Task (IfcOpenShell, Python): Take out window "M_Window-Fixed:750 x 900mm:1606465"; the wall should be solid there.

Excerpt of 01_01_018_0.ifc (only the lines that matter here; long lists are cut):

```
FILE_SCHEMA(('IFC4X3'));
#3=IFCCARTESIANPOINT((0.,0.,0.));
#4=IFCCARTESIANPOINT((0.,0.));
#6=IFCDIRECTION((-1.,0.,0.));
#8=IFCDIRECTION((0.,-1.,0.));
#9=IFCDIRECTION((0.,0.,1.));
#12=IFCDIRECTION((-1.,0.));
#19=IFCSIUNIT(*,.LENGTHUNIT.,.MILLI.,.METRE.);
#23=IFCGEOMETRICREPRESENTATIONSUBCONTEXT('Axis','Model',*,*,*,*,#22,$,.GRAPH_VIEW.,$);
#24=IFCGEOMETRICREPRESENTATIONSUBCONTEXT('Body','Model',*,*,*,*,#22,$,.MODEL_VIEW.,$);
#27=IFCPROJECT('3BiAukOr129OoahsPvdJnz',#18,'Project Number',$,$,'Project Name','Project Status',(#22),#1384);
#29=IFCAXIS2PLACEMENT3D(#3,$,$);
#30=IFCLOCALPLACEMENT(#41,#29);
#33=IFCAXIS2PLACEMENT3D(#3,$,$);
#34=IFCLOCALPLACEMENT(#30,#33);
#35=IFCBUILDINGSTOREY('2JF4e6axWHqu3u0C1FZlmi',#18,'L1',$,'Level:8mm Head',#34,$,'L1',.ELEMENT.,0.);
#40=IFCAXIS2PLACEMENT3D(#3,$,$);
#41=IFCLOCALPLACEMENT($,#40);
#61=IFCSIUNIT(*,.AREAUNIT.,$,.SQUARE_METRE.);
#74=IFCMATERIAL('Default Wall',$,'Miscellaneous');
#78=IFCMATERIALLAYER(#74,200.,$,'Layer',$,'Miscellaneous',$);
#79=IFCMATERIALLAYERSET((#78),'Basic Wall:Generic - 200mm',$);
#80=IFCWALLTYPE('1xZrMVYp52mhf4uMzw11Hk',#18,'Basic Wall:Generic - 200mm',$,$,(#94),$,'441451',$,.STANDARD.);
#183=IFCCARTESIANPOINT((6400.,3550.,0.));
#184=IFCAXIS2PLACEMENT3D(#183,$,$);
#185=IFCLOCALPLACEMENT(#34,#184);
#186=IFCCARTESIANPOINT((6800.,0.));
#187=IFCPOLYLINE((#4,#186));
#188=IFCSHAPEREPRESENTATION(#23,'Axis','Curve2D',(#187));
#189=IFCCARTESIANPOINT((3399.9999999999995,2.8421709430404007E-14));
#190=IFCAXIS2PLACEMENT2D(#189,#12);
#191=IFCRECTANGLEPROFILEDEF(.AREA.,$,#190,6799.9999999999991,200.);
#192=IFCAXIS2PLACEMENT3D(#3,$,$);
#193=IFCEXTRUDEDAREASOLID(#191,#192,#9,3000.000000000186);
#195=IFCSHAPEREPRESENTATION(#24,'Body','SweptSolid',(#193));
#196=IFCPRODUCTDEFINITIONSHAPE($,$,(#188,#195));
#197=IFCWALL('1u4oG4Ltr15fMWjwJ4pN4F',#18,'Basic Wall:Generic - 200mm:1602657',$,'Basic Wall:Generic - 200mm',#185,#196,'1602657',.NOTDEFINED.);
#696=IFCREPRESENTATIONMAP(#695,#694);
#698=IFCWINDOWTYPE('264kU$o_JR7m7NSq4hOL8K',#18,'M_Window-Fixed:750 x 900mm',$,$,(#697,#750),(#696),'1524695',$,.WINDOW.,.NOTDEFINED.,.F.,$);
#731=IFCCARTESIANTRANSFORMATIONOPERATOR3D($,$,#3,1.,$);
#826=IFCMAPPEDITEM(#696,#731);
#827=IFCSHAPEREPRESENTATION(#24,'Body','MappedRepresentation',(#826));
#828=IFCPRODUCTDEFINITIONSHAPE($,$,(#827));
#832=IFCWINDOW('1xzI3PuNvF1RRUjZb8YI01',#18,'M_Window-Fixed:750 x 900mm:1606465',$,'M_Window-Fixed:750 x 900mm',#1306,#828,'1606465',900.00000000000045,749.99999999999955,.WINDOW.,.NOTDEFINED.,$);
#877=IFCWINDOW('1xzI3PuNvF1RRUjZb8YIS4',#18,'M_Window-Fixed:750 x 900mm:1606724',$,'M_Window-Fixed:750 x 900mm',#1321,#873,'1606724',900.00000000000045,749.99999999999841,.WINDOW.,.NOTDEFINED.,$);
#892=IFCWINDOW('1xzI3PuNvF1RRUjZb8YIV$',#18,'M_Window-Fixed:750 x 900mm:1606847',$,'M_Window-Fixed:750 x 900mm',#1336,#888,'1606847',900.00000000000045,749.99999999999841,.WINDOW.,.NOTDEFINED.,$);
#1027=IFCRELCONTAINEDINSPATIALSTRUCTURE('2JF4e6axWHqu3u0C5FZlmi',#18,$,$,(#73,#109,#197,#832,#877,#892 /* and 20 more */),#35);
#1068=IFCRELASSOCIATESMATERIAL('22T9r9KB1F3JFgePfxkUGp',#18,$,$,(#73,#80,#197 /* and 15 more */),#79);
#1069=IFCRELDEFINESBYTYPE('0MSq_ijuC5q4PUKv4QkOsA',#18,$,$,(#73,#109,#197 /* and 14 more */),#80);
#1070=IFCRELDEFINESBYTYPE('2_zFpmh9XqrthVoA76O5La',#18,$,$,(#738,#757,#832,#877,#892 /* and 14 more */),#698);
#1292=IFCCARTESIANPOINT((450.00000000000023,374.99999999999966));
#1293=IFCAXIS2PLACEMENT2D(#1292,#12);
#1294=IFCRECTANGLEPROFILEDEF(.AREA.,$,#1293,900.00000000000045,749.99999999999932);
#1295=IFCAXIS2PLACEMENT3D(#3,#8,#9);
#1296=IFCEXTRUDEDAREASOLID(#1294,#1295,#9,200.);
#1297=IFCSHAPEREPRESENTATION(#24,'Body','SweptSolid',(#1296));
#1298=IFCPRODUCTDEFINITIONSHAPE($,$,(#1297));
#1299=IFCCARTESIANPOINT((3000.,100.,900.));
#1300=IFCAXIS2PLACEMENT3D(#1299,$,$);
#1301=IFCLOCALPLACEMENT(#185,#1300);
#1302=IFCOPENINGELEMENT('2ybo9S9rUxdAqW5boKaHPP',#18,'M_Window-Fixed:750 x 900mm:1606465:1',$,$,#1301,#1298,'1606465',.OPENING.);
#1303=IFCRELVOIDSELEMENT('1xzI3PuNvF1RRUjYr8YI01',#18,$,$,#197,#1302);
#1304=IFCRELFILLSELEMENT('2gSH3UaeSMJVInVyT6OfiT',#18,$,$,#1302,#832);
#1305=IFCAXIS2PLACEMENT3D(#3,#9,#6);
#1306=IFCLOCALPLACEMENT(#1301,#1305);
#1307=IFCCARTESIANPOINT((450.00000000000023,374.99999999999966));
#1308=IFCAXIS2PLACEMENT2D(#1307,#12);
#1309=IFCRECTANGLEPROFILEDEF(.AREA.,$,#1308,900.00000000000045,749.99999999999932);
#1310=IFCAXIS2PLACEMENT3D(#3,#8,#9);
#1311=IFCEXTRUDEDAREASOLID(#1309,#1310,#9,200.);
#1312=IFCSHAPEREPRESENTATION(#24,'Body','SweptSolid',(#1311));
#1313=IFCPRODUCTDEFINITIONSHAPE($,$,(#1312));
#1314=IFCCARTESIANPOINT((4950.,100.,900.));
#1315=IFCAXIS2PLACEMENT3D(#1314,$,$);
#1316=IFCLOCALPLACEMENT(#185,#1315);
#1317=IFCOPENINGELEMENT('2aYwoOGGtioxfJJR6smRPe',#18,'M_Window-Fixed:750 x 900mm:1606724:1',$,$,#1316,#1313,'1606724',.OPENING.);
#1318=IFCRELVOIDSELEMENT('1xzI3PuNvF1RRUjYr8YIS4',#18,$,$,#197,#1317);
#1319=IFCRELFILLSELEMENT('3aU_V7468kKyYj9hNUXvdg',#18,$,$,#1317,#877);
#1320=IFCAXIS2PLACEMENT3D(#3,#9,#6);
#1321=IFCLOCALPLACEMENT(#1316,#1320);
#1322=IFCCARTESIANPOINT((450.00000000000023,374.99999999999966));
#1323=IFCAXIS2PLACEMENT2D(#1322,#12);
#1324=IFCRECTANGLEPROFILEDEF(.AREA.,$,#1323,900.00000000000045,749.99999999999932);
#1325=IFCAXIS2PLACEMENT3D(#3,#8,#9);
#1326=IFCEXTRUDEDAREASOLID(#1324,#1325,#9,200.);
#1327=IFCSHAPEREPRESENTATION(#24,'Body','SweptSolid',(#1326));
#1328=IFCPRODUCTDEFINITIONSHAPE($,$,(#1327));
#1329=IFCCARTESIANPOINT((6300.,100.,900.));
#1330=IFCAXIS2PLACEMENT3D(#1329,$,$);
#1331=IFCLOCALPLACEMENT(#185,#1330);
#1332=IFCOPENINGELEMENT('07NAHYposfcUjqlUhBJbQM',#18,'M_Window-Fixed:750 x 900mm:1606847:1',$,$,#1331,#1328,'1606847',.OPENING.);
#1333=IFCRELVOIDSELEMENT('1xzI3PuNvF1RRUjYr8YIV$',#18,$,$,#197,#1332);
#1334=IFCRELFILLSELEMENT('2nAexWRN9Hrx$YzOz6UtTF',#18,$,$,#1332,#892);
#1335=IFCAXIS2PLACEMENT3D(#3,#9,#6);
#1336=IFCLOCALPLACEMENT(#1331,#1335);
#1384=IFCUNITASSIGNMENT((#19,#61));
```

```python
import ifcopenshell
import ifcopenshell.api.feature
import ifcopenshell.api.root
import ifcopenshell.geom
import ifcopenshell.util.shape

model = ifcopenshell.open("01_01_018_0.ifc")
settings = ifcopenshell.geom.settings()


def volume(element):
    """Net volume in cubic metres, openings subtracted."""
    shape = ifcopenshell.geom.create_shape(settings, element)
    return ifcopenshell.util.shape.get_volume(shape.geometry)


window = model.by_guid("1xzI3PuNvF1RRUjZb8YI01")
opening = window.FillsVoids[0].RelatingOpeningElement
wall = opening.VoidsElements[0].RelatingBuildingElement
before = volume(wall)

ifcopenshell.api.root.remove_product(model, product=window)
ifcopenshell.api.feature.remove_feature(model, feature=opening)

after = volume(wall)

print(f"wall volume {before:.3f} -> {after:.3f} m3")

model.write("01_01_018_0_rev.ifc")
```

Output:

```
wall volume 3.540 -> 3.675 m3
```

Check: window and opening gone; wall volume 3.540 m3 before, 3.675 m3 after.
